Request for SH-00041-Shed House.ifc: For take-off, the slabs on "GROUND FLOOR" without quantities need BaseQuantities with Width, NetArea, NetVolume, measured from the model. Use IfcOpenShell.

First a look at what the model holds.

```python
import ifcopenshell
import ifcopenshell.util.element
import ifcopenshell.util.unit

model = ifcopenshell.open("SH-00041-Shed House.ifc")
print(model.schema)
for unit_type in ("LENGTHUNIT", "AREAUNIT", "VOLUMEUNIT"):
    print(unit_type, ifcopenshell.util.unit.calculate_unit_scale(model, unit_type))
storey = next(s for s in model.by_type("IfcBuildingStorey") if s.Name == "GROUND FLOOR")
slabs = [e for e in ifcopenshell.util.element.get_decomposition(storey) if e.is_a("IfcSlab")]
for e in sorted(slabs, key=lambda e: e.id()):
    print(e.id(), e.is_a(), e.Name, list(ifcopenshell.util.element.get_psets(e, qtos_only=True)), sep=" | ")
```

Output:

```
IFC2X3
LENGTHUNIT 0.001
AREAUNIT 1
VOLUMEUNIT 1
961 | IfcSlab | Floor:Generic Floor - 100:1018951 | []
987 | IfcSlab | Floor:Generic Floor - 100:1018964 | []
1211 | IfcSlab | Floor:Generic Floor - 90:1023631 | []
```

```python
import ifcopenshell
import ifcopenshell.api.pset
import ifcopenshell.geom
import ifcopenshell.util.element
import ifcopenshell.util.shape
import ifcopenshell.util.unit

model = ifcopenshell.open("SH-00041-Shed House.ifc")
unit_scale = ifcopenshell.util.unit.calculate_unit_scale(model)
area_scale = ifcopenshell.util.unit.calculate_unit_scale(model, "AREAUNIT")
volume_scale = ifcopenshell.util.unit.calculate_unit_scale(model, "VOLUMEUNIT")
settings = ifcopenshell.geom.settings()

storey = next(s for s in model.by_type("IfcBuildingStorey") if s.Name == "GROUND FLOOR")
slabs = [e for e in ifcopenshell.util.element.get_decomposition(storey) if e.is_a("IfcSlab")]

for e in sorted(slabs, key=lambda e: e.id()):
    if ifcopenshell.util.element.get_psets(e, qtos_only=True, should_inherit=False):
        continue
    # Geometry comes back in metres, in the element's own axes.
    shape = ifcopenshell.geom.create_shape(settings, e)
    values = {
        "Width": ifcopenshell.util.shape.get_z(shape.geometry) / unit_scale,
        "NetArea": ifcopenshell.util.shape.get_footprint_area(shape.geometry) / area_scale,
        "NetVolume": ifcopenshell.util.shape.get_volume(shape.geometry) / volume_scale,
    }
    qto = ifcopenshell.api.pset.add_qto(model, product=e, name="BaseQuantities")
    ifcopenshell.api.pset.edit_qto(model, qto=qto, properties=values)
    print(e.id(), {k: round(v, 3) for k, v in values.items()})

model.write("SH-00041-Shed House_v2.ifc")
```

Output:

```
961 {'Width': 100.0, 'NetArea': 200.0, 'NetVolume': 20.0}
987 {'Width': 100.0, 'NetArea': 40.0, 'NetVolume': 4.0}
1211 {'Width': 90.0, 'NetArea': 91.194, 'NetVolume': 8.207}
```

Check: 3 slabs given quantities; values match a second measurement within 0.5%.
